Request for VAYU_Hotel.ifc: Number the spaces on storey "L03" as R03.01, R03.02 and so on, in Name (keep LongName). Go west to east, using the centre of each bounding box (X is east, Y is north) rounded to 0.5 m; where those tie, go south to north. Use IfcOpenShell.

First a look at what the model holds.

```python
import ifcopenshell
import ifcopenshell.util.element
import ifcopenshell.util.placement

model = ifcopenshell.open("VAYU_Hotel.ifc")
print(model.schema)
storey = next(s for s in model.by_type("IfcBuildingStorey") if s.Name == "L03")
spaces = [e for e in ifcopenshell.util.element.get_decomposition(storey) if e.is_a("IfcSpace")]
for e in sorted(spaces, key=lambda e: e.id()):
    origin = ifcopenshell.util.placement.get_local_placement(e.ObjectPlacement)[:3, 3]
    print(e.id(), e.Name, e.LongName, origin.round(2) + 0.0, sep=" | ")
```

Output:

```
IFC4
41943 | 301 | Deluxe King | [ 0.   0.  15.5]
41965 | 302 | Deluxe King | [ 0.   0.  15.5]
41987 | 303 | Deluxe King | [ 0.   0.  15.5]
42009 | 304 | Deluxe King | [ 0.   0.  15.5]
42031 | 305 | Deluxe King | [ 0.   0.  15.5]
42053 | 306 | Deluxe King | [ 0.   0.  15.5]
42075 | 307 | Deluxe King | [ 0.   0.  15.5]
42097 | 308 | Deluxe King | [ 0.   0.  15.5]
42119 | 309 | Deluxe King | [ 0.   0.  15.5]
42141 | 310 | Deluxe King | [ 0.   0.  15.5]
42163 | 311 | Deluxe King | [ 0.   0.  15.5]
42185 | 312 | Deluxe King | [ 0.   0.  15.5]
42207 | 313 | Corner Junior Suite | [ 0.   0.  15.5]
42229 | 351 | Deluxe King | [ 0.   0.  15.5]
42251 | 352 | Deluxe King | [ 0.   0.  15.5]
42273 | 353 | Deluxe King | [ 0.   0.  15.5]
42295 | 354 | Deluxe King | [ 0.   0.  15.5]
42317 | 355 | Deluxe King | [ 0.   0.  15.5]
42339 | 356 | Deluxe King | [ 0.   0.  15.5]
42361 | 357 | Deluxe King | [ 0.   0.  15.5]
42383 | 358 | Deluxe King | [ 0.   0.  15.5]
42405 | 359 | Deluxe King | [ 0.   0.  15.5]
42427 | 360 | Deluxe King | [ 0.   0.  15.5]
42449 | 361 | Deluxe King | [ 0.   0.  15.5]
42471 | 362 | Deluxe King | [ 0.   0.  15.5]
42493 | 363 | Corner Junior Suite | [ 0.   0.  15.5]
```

```python
import ifcopenshell
import ifcopenshell.geom
import ifcopenshell.util.element
import ifcopenshell.util.shape

model = ifcopenshell.open("VAYU_Hotel.ifc")
settings = ifcopenshell.geom.settings()
settings.set("use-world-coords", True)


def centre(element):
    shape = ifcopenshell.geom.create_shape(settings, element)
    return ifcopenshell.util.shape.get_bbox_centroid(shape.geometry)


storey = next(s for s in model.by_type("IfcBuildingStorey") if s.Name == "L03")
spaces = [e for e in ifcopenshell.util.element.get_decomposition(storey) if e.is_a("IfcSpace")]

# Insertion points can sit at a corner or the storey origin, so sort by the geometry (in metres).
centres = {e: centre(e) for e in spaces}
spaces.sort(key=lambda e: (round(centres[e][0] / 0.5), centres[e][1]))

for i, e in enumerate(spaces, start=1):
    number = f"R03.{i:02d}"
    e.Name = number
    print(e.id(), number)

model.write("VAYU_Hotel_v2.ifc")
```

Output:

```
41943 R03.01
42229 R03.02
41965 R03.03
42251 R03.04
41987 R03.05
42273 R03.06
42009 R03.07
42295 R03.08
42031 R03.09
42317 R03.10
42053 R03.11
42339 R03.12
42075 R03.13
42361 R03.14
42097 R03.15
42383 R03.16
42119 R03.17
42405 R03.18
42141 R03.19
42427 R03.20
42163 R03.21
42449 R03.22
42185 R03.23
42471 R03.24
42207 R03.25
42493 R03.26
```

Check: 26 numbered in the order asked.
